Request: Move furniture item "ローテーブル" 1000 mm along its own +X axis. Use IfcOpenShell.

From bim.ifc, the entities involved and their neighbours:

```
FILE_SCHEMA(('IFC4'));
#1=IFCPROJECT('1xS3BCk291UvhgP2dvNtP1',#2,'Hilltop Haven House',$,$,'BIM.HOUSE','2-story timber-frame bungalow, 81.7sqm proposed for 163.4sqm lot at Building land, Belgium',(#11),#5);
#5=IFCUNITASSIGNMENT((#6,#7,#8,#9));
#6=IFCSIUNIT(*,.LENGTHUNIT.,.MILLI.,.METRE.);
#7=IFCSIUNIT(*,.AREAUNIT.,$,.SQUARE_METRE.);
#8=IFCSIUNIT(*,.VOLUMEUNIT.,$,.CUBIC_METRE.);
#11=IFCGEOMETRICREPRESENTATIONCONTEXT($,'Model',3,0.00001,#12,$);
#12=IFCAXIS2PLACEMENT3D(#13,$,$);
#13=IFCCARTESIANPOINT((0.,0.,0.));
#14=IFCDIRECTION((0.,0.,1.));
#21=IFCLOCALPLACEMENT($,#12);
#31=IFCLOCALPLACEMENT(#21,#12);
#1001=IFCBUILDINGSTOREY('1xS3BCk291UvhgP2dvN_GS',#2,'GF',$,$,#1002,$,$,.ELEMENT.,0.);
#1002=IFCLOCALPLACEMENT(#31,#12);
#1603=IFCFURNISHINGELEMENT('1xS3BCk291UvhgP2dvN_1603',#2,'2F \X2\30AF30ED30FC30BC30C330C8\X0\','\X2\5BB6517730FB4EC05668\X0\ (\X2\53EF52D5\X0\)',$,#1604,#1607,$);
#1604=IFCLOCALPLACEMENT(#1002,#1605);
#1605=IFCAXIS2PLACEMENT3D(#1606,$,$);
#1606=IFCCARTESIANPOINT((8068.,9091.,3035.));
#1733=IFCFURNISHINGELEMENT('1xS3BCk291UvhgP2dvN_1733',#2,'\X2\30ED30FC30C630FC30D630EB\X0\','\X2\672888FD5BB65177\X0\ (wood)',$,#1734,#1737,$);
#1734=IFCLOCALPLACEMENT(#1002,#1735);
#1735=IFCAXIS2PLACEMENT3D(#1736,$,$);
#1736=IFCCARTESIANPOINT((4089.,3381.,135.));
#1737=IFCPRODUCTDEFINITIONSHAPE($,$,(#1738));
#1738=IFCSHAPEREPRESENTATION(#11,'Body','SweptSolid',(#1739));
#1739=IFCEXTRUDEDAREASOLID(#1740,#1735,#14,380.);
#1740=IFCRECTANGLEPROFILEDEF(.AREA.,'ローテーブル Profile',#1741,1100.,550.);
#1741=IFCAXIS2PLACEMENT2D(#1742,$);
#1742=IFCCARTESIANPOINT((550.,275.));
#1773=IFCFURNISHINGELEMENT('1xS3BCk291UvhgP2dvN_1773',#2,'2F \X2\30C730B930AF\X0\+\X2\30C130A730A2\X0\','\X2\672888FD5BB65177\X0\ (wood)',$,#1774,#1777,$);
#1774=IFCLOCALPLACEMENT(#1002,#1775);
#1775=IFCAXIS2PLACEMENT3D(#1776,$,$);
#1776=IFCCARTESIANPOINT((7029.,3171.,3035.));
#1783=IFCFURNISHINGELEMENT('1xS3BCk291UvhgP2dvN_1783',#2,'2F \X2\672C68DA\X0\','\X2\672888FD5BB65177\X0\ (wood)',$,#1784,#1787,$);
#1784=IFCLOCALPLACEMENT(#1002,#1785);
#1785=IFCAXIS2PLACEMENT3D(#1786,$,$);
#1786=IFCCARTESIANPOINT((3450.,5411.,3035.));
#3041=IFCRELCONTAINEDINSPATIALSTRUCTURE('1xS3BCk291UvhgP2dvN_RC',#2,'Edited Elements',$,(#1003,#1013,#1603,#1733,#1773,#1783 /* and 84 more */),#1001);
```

```python
import ifcopenshell
import ifcopenshell.api.geometry
import ifcopenshell.util.placement
import ifcopenshell.util.unit

model = ifcopenshell.open("bim.ifc")
unit_scale = ifcopenshell.util.unit.calculate_unit_scale(model)

item = model.by_guid("1xS3BCk291UvhgP2dvN_1733")
matrix = ifcopenshell.util.placement.get_local_placement(item.ObjectPlacement)
matrix[:3, 3] += matrix[:3, 0] * 1 / unit_scale
ifcopenshell.api.geometry.edit_object_placement(model, product=item, matrix=matrix, is_si=False)

print(ifcopenshell.util.placement.get_local_placement(item.ObjectPlacement).round(3) + 0.0)

model.write("bim_v2.ifc")
```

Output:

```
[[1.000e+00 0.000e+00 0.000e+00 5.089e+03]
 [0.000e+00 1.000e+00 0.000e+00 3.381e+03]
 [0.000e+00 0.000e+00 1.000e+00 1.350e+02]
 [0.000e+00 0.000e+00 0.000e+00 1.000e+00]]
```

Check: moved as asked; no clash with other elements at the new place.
